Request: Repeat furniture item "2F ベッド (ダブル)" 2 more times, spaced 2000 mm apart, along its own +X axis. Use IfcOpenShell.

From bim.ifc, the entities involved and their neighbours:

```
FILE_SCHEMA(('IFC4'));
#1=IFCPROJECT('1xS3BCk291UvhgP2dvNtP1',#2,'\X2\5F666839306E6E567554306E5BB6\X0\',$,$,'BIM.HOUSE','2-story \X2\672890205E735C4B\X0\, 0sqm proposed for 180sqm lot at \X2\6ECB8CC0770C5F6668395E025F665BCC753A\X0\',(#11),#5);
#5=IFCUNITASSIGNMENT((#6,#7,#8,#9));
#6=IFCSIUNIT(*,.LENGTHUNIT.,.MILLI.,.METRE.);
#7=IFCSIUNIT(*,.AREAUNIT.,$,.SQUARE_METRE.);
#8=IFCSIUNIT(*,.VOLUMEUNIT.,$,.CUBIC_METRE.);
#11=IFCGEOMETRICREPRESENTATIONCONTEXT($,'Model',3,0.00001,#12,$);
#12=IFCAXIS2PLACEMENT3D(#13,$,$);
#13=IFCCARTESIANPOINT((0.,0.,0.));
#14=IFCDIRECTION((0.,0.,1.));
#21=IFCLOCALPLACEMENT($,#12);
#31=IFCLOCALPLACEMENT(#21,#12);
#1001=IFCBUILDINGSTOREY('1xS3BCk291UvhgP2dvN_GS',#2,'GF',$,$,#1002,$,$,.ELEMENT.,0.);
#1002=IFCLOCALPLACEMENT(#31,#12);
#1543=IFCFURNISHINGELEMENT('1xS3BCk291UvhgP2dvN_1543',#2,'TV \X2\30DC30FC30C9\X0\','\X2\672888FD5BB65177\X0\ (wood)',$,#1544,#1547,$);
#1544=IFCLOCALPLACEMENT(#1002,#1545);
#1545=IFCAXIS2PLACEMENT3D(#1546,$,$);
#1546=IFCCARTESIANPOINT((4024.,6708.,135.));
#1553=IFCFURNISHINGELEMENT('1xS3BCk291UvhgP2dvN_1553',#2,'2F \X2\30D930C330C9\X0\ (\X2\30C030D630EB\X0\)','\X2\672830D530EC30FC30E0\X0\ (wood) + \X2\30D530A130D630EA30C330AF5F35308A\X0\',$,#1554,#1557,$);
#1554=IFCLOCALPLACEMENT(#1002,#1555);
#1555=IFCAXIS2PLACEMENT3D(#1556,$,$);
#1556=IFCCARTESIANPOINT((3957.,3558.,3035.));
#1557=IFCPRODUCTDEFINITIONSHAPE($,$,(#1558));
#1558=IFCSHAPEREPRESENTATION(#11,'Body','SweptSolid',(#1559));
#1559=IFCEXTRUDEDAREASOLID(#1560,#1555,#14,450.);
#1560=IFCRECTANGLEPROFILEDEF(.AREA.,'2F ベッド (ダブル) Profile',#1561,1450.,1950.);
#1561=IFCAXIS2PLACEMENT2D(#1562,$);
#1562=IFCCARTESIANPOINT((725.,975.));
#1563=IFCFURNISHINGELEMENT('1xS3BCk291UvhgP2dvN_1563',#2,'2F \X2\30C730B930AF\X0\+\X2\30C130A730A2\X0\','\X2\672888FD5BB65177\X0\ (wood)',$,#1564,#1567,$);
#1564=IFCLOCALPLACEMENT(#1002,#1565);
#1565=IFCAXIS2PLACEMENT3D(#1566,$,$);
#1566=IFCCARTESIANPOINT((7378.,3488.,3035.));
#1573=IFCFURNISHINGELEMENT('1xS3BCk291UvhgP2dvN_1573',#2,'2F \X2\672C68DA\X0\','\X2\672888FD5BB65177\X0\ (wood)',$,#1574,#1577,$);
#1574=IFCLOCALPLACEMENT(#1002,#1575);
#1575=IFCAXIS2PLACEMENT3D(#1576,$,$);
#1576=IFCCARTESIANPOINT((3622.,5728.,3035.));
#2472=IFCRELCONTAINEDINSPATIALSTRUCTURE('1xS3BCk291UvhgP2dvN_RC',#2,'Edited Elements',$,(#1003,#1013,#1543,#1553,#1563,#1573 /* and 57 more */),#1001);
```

```python
import ifcopenshell
import ifcopenshell.api.geometry
import ifcopenshell.api.root
import ifcopenshell.util.element
import ifcopenshell.util.placement

model = ifcopenshell.open("bim.ifc")


def reuse_history(source, copy):
    """copy_class also copies each property set's owner history, people and application; keep the originals."""
    for rel in copy.IsDefinedBy:
        if rel.is_a("IfcRelDefinesByProperties") and (history := rel.RelatingPropertyDefinition.OwnerHistory):
            rel.RelatingPropertyDefinition.OwnerHistory = source.OwnerHistory
            ifcopenshell.util.element.remove_deep2(model, history)


source = model.by_guid("1xS3BCk291UvhgP2dvN_1553")
base = ifcopenshell.util.placement.get_local_placement(source.ObjectPlacement)
step = base[:3, 0] * 2000.0

for i in range(1, 3):
    copy = ifcopenshell.api.root.copy_class(model, product=source)
    copy.Representation = ifcopenshell.util.element.copy_deep(
        model, source.Representation, exclude=["IfcGeometricRepresentationContext", "IfcRepresentationMap"]
    )
    reuse_history(source, copy)
    matrix = base.copy()
    matrix[:3, 3] += i * step
    print("added at", matrix[:3, 3].round(3) + 0.0)
    ifcopenshell.api.geometry.edit_object_placement(model, product=copy, matrix=matrix, is_si=False)

model.write("bim_updated.ifc")
```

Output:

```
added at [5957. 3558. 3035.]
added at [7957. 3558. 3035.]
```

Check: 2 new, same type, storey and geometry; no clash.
